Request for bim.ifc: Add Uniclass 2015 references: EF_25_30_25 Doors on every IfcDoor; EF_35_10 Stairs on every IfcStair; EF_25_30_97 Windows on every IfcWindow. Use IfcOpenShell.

First a look at what the model holds.

```python
import ifcopenshell

model = ifcopenshell.open("bim.ifc")
print(model.schema)
print("classifications:", [c.Name for c in model.by_type("IfcClassification")])
for ifc_class in ("IfcDoor", "IfcRoof", "IfcStair", "IfcWall", "IfcWindow"):
    print(ifc_class, len(model.by_type(ifc_class)))
```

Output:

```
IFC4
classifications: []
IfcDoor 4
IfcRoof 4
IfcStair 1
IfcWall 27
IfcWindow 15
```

```python
import ifcopenshell
import ifcopenshell.api.classification

model = ifcopenshell.open("bim.ifc")

system = ifcopenshell.api.classification.add_classification(model, classification="Uniclass 2015")

codes = {
    "IfcDoor": ("EF_25_30_25", "Doors"),
    "IfcStair": ("EF_35_10", "Stairs"),
    "IfcWindow": ("EF_25_30_97", "Windows"),
}
for ifc_class, (code, name) in codes.items():
    products = model.by_type(ifc_class)
    ifcopenshell.api.classification.add_reference(
        model, products=products, classification=system, identification=code, name=name
    )
    print(code, len(products))

model.write("bim_updated.ifc")
```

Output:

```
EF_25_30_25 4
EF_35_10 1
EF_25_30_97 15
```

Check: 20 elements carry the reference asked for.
